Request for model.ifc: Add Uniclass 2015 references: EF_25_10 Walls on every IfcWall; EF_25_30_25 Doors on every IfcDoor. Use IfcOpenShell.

First a look at what the model holds.

```python
import ifcopenshell

model = ifcopenshell.open("model.ifc")
print(model.schema)
print("classifications:", [c.Name for c in model.by_type("IfcClassification")])
for ifc_class in ("IfcDoor", "IfcRoof", "IfcStair", "IfcWall", "IfcWindow"):
    print(ifc_class, len(model.by_type(ifc_class)))
```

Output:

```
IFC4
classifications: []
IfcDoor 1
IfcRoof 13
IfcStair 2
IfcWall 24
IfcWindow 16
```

```python
import ifcopenshell
import ifcopenshell.api.classification

model = ifcopenshell.open("model.ifc")

system = ifcopenshell.api.classification.add_classification(model, classification="Uniclass 2015")

codes = {
    "IfcWall": ("EF_25_10", "Walls"),
    "IfcDoor": ("EF_25_30_25", "Doors"),
}
for ifc_class, (code, name) in codes.items():
    products = model.by_type(ifc_class)
    ifcopenshell.api.classification.add_reference(
        model, products=products, classification=system, identification=code, name=name
    )
    print(code, len(products))

model.write("model_updated.ifc")
```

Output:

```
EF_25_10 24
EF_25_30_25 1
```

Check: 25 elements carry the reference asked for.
